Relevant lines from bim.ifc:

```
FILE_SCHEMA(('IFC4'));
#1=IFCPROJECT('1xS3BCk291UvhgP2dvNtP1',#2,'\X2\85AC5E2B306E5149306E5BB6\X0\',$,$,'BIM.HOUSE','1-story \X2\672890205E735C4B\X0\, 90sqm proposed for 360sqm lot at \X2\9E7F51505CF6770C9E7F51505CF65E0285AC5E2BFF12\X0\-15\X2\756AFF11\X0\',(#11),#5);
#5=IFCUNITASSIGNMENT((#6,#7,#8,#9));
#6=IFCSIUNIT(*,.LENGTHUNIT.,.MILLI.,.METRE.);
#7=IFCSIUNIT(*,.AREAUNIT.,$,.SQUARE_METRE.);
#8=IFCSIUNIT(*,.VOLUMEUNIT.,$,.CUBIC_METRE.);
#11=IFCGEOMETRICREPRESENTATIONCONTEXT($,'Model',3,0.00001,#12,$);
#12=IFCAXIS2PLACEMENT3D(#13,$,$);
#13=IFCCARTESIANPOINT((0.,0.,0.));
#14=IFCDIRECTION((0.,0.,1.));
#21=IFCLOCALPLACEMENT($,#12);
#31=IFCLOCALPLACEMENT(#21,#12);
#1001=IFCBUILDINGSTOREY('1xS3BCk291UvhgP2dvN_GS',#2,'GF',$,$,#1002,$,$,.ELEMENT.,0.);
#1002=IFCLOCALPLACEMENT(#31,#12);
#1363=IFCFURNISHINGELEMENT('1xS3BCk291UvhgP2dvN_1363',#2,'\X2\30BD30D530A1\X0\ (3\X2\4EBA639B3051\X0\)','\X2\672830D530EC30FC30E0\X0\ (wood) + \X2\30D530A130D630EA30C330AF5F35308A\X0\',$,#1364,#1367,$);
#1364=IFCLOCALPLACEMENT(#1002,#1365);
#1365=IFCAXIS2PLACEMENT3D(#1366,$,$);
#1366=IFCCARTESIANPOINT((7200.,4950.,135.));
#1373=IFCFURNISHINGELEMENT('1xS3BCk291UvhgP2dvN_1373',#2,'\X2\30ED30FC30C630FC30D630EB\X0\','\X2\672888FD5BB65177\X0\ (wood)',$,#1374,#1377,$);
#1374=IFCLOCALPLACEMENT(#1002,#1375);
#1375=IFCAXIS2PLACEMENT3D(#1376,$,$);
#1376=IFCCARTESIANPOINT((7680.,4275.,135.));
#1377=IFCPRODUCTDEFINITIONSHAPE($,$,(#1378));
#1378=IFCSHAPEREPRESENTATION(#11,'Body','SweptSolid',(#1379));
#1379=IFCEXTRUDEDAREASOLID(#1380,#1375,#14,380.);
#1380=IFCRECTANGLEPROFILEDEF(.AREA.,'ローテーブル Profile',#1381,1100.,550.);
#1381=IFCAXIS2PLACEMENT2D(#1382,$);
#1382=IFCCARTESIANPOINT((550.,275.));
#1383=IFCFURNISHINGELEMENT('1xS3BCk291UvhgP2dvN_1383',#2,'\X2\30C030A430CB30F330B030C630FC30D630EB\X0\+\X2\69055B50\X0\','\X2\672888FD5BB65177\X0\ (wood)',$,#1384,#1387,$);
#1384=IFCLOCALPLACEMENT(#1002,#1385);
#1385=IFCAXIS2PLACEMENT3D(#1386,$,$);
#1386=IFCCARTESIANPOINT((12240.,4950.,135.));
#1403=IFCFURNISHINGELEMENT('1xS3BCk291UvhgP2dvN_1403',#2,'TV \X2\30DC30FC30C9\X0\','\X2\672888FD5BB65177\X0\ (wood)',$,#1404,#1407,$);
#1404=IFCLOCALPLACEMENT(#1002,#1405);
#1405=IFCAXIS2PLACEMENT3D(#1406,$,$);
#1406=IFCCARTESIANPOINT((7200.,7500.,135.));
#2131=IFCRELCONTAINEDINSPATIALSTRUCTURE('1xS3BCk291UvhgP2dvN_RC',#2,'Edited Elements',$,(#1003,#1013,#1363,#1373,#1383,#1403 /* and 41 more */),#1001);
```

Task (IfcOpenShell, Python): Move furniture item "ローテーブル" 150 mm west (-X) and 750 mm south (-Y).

```python
import ifcopenshell
import ifcopenshell.api.geometry
import ifcopenshell.util.placement
import ifcopenshell.util.unit

model = ifcopenshell.open("bim.ifc")
unit_scale = ifcopenshell.util.unit.calculate_unit_scale(model)

item = model.by_id(1373)
matrix = ifcopenshell.util.placement.get_local_placement(item.ObjectPlacement)
matrix[0, 3] -= 0.15 / unit_scale
matrix[1, 3] -= 0.75 / unit_scale
ifcopenshell.api.geometry.edit_object_placement(model, product=item, matrix=matrix, is_si=False)

print(ifcopenshell.util.placement.get_local_placement(item.ObjectPlacement).round(3) + 0.0)

model.write("bim_rev.ifc")
```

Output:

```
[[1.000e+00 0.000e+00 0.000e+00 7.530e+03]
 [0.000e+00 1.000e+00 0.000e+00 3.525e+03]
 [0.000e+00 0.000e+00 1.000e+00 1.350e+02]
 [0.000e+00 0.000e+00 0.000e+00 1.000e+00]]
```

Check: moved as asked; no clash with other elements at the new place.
